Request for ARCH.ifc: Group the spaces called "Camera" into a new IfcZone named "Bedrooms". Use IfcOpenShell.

First a look at what the model holds.

```python
import ifcopenshell

model = ifcopenshell.open("ARCH.ifc")
print(model.schema)
seen = {}
for space in model.by_type("IfcSpace"):
    seen[space.LongName] = seen.get(space.LongName, 0) + 1
for name, count in sorted(seen.items(), key=str):
    print(count, "x", name)
print("zones:", [z.Name for z in model.by_type("IfcZone")][:20])
```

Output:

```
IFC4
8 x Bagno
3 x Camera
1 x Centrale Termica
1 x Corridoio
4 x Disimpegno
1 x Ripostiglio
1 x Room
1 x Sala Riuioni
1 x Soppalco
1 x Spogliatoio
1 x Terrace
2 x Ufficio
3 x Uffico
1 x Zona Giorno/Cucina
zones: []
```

```python
import ifcopenshell
import ifcopenshell.api.group
import ifcopenshell.api.root

model = ifcopenshell.open("ARCH.ifc")

names = {"Camera"}
spaces = [s for s in model.by_type("IfcSpace") if s.LongName in names]

zone = ifcopenshell.api.root.create_entity(model, ifc_class="IfcZone", name="Bedrooms")
ifcopenshell.api.group.assign_group(model, products=spaces, group=zone)
print(len(spaces), "spaces in", zone.Name)

model.write("ARCH_v2.ifc")
```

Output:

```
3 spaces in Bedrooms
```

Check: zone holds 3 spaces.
